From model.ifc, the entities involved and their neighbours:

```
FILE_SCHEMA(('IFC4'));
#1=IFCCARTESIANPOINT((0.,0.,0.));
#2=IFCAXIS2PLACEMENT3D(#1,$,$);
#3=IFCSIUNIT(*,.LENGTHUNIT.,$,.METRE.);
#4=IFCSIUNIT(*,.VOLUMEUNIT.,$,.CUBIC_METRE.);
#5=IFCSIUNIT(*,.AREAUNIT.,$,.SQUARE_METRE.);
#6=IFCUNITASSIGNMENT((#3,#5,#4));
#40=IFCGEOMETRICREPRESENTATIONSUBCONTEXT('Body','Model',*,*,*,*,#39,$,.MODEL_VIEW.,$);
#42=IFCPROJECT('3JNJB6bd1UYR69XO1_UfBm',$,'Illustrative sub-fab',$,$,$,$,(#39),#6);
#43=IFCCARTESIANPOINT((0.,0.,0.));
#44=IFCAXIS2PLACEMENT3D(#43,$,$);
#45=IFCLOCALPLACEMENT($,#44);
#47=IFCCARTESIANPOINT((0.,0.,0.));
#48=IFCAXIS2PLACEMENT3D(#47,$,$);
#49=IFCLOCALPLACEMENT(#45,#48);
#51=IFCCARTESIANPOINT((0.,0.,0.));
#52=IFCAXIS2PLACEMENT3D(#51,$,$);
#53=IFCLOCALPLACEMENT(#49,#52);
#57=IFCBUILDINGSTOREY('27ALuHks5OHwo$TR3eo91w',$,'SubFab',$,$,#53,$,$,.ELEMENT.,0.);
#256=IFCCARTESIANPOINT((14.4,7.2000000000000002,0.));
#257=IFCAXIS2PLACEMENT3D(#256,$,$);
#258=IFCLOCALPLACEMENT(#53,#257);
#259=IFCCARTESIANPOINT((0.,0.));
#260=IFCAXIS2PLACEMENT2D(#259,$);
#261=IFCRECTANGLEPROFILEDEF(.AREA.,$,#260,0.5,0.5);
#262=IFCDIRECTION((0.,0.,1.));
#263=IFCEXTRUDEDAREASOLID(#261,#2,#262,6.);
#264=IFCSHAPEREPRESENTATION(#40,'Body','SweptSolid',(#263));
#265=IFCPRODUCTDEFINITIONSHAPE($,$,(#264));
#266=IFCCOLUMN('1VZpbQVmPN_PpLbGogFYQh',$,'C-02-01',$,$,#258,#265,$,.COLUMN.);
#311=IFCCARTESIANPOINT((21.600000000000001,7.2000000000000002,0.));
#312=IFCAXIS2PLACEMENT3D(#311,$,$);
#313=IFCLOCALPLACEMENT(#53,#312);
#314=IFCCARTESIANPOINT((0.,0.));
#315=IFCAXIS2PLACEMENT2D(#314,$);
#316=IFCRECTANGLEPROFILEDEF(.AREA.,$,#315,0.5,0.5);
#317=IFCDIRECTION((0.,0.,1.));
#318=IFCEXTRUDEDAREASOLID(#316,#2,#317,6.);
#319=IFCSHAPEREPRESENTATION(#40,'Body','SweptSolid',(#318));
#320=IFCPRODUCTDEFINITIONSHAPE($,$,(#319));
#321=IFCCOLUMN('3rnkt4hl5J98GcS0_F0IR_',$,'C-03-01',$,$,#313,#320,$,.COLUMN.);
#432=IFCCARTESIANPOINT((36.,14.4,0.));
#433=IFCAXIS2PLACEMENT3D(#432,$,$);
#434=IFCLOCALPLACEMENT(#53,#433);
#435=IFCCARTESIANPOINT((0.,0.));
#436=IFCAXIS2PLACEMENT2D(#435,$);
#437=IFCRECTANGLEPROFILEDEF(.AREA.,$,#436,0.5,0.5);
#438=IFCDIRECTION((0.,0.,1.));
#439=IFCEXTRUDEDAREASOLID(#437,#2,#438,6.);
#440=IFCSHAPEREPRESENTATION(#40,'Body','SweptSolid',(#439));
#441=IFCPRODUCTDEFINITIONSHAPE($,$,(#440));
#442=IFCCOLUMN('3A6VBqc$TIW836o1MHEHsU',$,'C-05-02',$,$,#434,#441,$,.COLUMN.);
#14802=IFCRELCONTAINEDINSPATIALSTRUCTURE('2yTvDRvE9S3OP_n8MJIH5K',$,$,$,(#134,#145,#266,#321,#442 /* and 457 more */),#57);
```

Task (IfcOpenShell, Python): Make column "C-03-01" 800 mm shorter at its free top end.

```python
import ifcopenshell
import ifcopenshell.util.representation

model = ifcopenshell.open("model.ifc")

member = model.by_guid("3rnkt4hl5J98GcS0_F0IR_")
change = -0.8

# The extrusion runs towards the end named, so only its depth changes.
body = ifcopenshell.util.representation.get_representation(member, "Model", "Body")
solid = body.Items[0]
old_length = solid.Depth
solid.Depth += change

print(f"length {old_length:g} -> {solid.Depth:g}")

model.write("model_rev.ifc")
```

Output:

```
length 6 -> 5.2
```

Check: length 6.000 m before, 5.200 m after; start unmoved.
